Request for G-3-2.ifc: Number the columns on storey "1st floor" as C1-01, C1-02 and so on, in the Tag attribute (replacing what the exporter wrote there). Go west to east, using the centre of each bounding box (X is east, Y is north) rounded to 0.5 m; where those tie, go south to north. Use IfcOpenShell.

First a look at what the model holds.

```python
import ifcopenshell
import ifcopenshell.util.element
import ifcopenshell.util.placement

model = ifcopenshell.open("G-3-2.ifc")
print(model.schema)
storey = next(s for s in model.by_type("IfcBuildingStorey") if s.Name == "1st floor")
columns = [e for e in ifcopenshell.util.element.get_decomposition(storey) if e.is_a("IfcColumn")]
for e in sorted(columns, key=lambda e: e.id()):
    origin = ifcopenshell.util.placement.get_local_placement(e.ObjectPlacement)[:3, 3]
    print(e.id(), e.Tag, e.Name, origin.round(2) + 0.0, sep=" | ")
```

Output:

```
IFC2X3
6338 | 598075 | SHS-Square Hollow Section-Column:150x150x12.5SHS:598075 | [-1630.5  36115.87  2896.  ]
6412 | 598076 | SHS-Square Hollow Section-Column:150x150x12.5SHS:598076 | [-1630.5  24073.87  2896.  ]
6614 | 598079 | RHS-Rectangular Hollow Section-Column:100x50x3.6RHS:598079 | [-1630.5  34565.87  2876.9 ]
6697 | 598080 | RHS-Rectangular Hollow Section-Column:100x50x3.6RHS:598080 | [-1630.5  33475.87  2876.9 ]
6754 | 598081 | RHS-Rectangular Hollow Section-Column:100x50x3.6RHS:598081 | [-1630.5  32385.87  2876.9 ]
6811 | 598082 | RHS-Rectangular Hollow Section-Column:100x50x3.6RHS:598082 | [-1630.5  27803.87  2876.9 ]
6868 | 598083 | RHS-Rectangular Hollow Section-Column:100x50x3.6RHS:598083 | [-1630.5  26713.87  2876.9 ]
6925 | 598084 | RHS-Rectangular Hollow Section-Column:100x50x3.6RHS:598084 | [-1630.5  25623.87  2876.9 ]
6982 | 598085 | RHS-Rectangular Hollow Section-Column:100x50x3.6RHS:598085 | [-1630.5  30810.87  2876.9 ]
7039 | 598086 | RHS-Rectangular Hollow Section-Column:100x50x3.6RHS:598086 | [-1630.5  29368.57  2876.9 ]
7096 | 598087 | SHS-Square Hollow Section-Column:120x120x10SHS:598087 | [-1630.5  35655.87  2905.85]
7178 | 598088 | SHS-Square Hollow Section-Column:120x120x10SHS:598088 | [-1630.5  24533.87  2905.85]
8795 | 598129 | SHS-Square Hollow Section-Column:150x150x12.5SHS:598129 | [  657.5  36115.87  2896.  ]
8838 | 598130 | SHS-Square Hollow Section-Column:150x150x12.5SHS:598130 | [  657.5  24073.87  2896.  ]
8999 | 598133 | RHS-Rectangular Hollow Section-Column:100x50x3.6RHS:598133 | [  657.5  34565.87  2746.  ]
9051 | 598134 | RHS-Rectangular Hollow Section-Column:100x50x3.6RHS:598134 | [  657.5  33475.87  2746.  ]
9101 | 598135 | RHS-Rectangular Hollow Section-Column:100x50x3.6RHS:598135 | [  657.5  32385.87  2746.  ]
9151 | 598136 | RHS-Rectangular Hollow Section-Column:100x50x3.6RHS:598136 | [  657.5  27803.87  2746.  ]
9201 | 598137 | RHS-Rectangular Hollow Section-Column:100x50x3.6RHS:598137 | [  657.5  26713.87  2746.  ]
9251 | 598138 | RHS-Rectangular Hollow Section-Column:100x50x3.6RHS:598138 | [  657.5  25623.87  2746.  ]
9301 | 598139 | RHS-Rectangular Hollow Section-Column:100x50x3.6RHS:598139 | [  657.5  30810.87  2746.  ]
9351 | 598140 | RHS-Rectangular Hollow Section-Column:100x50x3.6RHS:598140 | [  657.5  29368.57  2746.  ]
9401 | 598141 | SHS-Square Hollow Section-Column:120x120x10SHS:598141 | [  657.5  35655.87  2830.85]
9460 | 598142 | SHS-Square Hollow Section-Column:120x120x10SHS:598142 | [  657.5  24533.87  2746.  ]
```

```python
import ifcopenshell
import ifcopenshell.geom
import ifcopenshell.util.element
import ifcopenshell.util.shape

model = ifcopenshell.open("G-3-2.ifc")
settings = ifcopenshell.geom.settings()
settings.set("use-world-coords", True)


def centre(element):
    shape = ifcopenshell.geom.create_shape(settings, element)
    return ifcopenshell.util.shape.get_bbox_centroid(shape.geometry)


storey = next(s for s in model.by_type("IfcBuildingStorey") if s.Name == "1st floor")
columns = [e for e in ifcopenshell.util.element.get_decomposition(storey) if e.is_a("IfcColumn")]

# Insertion points can sit at a corner or the storey origin, so sort by the geometry (in metres).
centres = {e: centre(e) for e in columns}
columns.sort(key=lambda e: (round(centres[e][0] / 0.5), centres[e][1]))

for i, e in enumerate(columns, start=1):
    number = f"C1-{i:02d}"
    e.Tag = number
    print(e.id(), number)

model.write("G-3-2-out.ifc")
```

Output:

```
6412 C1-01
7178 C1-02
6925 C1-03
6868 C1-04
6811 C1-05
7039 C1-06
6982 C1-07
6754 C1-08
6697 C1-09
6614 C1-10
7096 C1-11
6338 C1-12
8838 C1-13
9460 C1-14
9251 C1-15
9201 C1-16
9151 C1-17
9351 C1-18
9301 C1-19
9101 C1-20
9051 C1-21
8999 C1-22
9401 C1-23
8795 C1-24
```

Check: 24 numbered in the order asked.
